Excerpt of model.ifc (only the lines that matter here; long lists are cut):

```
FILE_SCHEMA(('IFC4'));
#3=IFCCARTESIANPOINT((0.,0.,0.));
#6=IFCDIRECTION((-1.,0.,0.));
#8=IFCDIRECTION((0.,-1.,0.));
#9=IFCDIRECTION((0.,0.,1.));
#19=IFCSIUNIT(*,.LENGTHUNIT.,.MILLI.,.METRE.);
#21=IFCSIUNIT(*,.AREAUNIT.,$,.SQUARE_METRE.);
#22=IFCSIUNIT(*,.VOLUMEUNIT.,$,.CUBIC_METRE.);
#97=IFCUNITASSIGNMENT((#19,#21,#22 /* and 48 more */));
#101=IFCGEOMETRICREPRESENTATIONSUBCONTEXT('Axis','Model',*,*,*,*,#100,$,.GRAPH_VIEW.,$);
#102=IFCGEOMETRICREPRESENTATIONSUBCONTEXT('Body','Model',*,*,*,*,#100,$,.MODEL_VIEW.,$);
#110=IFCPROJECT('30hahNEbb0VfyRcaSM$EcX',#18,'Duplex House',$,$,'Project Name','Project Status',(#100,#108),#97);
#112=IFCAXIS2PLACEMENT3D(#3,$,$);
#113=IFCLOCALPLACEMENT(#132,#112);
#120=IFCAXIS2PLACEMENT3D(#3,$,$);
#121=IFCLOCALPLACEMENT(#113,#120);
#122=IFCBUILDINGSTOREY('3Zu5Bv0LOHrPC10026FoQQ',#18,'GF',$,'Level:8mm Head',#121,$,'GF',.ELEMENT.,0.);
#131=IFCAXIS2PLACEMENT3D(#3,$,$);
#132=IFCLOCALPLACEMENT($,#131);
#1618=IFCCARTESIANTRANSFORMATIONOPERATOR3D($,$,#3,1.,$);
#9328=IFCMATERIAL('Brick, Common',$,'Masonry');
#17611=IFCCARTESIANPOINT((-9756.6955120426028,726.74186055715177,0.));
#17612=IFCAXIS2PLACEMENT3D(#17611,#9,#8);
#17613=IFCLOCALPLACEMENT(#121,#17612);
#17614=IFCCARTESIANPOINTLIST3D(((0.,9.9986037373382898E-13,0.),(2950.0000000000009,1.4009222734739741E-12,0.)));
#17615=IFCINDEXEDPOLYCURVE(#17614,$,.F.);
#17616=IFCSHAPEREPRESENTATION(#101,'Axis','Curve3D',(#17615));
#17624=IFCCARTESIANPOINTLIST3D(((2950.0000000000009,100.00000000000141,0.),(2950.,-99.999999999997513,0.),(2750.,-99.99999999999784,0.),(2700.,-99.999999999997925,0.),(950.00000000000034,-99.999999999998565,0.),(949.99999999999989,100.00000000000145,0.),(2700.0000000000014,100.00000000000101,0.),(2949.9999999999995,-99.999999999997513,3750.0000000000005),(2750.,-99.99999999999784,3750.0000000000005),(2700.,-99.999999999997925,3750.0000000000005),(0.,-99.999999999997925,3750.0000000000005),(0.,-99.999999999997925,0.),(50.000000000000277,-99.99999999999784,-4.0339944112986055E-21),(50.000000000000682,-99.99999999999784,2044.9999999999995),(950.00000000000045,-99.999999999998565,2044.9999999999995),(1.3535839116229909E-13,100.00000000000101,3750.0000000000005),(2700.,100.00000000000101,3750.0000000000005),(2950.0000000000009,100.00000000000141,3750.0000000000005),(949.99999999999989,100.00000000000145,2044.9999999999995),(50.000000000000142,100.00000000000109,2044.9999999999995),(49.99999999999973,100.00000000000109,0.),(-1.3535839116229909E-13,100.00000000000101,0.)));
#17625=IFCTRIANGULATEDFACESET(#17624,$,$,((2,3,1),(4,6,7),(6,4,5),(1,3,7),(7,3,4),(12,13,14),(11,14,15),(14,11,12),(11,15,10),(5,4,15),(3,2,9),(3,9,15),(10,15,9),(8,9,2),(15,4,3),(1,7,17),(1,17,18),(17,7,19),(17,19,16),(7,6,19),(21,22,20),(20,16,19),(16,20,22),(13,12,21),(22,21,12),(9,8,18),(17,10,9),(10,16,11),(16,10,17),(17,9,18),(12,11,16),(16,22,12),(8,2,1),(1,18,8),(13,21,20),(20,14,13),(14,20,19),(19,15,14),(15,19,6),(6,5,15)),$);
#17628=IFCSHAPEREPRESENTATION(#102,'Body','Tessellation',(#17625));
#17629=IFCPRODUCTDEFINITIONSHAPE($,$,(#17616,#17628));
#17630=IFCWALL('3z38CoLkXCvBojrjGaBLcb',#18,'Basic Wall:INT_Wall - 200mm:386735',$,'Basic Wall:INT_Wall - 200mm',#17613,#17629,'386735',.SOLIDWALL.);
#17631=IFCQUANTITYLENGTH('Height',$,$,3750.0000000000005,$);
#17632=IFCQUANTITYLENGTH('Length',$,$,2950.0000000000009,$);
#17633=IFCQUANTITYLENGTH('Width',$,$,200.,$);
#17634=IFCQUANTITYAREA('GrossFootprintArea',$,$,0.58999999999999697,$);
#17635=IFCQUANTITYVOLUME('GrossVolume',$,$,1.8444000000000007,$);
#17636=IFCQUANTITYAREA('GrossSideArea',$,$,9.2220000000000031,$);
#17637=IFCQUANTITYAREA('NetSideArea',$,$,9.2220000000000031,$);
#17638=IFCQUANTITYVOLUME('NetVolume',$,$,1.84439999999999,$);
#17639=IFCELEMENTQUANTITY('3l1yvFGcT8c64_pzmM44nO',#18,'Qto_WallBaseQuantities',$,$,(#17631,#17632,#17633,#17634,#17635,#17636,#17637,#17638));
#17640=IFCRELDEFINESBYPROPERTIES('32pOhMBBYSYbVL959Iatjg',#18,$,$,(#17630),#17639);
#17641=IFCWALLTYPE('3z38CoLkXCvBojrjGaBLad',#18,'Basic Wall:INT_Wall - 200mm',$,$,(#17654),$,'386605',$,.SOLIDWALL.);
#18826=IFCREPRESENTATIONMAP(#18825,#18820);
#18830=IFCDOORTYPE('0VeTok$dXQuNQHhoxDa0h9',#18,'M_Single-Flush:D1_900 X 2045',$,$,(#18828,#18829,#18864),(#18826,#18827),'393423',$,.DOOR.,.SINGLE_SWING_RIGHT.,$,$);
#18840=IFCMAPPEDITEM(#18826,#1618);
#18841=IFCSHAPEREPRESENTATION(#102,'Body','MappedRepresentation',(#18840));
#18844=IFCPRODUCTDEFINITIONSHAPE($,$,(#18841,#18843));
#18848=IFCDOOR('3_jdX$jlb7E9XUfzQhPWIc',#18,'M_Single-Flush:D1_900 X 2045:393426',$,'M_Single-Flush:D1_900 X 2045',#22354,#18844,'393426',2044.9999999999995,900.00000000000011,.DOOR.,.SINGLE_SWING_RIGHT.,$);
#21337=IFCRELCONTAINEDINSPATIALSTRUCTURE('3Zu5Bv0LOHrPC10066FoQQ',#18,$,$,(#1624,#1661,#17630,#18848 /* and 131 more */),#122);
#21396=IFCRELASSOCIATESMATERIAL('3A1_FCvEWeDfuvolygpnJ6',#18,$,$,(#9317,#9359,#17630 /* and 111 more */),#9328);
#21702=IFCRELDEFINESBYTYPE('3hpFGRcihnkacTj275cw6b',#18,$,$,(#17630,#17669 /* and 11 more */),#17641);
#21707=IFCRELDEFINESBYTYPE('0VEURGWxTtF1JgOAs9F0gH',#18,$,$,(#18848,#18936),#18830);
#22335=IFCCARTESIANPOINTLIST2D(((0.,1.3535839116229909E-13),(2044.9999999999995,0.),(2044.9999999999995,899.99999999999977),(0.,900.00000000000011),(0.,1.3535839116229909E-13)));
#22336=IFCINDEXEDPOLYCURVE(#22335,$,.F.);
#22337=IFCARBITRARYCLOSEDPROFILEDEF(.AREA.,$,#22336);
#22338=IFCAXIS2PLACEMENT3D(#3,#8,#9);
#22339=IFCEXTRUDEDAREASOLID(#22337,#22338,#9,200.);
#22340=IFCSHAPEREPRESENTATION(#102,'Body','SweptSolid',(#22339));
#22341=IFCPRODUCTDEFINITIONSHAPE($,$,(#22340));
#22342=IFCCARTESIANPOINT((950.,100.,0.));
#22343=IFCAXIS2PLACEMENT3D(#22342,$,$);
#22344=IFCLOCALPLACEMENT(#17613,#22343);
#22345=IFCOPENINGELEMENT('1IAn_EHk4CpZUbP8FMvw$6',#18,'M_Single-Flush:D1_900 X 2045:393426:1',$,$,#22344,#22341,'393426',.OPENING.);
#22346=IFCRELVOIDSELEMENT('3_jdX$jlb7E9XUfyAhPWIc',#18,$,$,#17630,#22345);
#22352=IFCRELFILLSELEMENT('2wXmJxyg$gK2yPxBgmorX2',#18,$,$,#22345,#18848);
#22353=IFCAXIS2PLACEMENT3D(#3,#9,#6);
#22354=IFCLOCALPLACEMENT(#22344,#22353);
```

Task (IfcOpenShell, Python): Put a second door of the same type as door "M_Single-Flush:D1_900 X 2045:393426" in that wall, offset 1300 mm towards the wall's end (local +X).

```python
import ifcopenshell
import ifcopenshell.api.feature
import ifcopenshell.api.geometry
import ifcopenshell.api.pset
import ifcopenshell.api.root
import ifcopenshell.geom
import ifcopenshell.util.element
import ifcopenshell.util.placement
import ifcopenshell.util.shape
import ifcopenshell.util.unit

model = ifcopenshell.open("model.ifc")
unit_scale = ifcopenshell.util.unit.calculate_unit_scale(model)
area_scale = ifcopenshell.util.unit.calculate_unit_scale(model, "AREAUNIT")
volume_scale = ifcopenshell.util.unit.calculate_unit_scale(model, "VOLUMEUNIT")
settings = ifcopenshell.geom.settings()


def volume(element):
    """Net volume in cubic metres, openings subtracted."""
    shape = ifcopenshell.geom.create_shape(settings, element)
    return ifcopenshell.util.shape.get_volume(shape.geometry)


def reuse_history(source, copy):
    """copy_class also copies each property set's owner history, people and application; keep the originals."""
    for rel in copy.IsDefinedBy:
        if rel.is_a("IfcRelDefinesByProperties") and (history := rel.RelatingPropertyDefinition.OwnerHistory):
            rel.RelatingPropertyDefinition.OwnerHistory = source.OwnerHistory
            ifcopenshell.util.element.remove_deep2(model, history)


door = model.by_id(18848)
opening = door.FillsVoids[0].RelatingOpeningElement
wall = opening.VoidsElements[0].RelatingBuildingElement
before = volume(wall)
shift = ifcopenshell.util.placement.get_local_placement(wall.ObjectPlacement)[:3, 0] * 1.3 / unit_scale

# copy_class copies the void relationship, type, container and properties, but no geometry.
new_opening = ifcopenshell.api.root.copy_class(model, product=opening)
new_opening.Representation = ifcopenshell.util.element.copy_deep(
    model, opening.Representation, exclude=["IfcGeometricRepresentationContext", "IfcRepresentationMap"]
)
new_opening.Name = "M_Single-Flush:D1_900 X 2045"
new_opening.Tag = None
reuse_history(opening, new_opening)
new_door = ifcopenshell.api.root.copy_class(model, product=door)
new_door.Representation = ifcopenshell.util.element.copy_deep(
    model, door.Representation, exclude=["IfcGeometricRepresentationContext", "IfcRepresentationMap"]
)
new_door.Name = "M_Single-Flush:D1_900 X 2045"
new_door.Tag = None
reuse_history(door, new_door)
ifcopenshell.api.feature.add_filling(model, opening=new_opening, element=new_door)

for old, new in ((opening, new_opening), (door, new_door)):
    matrix = ifcopenshell.util.placement.get_local_placement(old.ObjectPlacement)
    matrix[:3, 3] += shift
    ifcopenshell.api.geometry.edit_object_placement(model, product=new, matrix=matrix, is_si=False)

after = volume(wall)
thickness = 0.2  # wall thickness in metres

# Update the wall's stored quantities.
qto = model.by_id(ifcopenshell.util.element.get_pset(wall, "Qto_WallBaseQuantities", should_inherit=False)["id"])
ifcopenshell.api.pset.edit_qto(model, qto=qto, properties={
    "NetSideArea": after / thickness / area_scale,
    "NetVolume": after / volume_scale,
})

print(f"wall volume {before:.3f} -> {after:.3f} m3")

model.write("model-out.ifc")
```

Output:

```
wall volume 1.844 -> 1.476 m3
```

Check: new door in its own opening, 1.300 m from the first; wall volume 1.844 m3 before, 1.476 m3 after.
